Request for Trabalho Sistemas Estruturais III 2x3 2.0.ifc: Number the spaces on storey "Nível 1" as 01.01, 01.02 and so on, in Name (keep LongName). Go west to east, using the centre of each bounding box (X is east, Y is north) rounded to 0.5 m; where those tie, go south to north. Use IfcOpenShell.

First a look at what the model holds.

```python
import ifcopenshell
import ifcopenshell.util.element
import ifcopenshell.util.placement

model = ifcopenshell.open("Trabalho Sistemas Estruturais III 2x3 2.0.ifc")
print(model.schema)
storey = next(s for s in model.by_type("IfcBuildingStorey") if s.Name == "Nível 1")
spaces = [e for e in ifcopenshell.util.element.get_decomposition(storey) if e.is_a("IfcSpace")]
for e in sorted(spaces, key=lambda e: e.id()):
    origin = ifcopenshell.util.placement.get_local_placement(e.ObjectPlacement)[:3, 3]
    print(e.id(), e.Name, e.LongName, origin.round(2) + 0.0, sep=" | ")
```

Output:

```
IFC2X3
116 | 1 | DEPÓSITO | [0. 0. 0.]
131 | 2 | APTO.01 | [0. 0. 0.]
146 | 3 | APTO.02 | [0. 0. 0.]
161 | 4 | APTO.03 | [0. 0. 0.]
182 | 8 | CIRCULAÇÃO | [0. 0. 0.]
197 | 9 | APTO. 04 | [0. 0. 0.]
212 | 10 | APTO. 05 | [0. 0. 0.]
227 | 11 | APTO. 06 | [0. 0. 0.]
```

```python
import ifcopenshell
import ifcopenshell.geom
import ifcopenshell.util.element
import ifcopenshell.util.shape

model = ifcopenshell.open("Trabalho Sistemas Estruturais III 2x3 2.0.ifc")
settings = ifcopenshell.geom.settings()
settings.set("use-world-coords", True)


def centre(element):
    shape = ifcopenshell.geom.create_shape(settings, element)
    return ifcopenshell.util.shape.get_bbox_centroid(shape.geometry)


storey = next(s for s in model.by_type("IfcBuildingStorey") if s.Name == "Nível 1")
spaces = [e for e in ifcopenshell.util.element.get_decomposition(storey) if e.is_a("IfcSpace")]

# Insertion points can sit at a corner or the storey origin, so sort by the geometry (in metres).
centres = {e: centre(e) for e in spaces}
spaces.sort(key=lambda e: (round(centres[e][0] / 0.5), centres[e][1]))

for i, e in enumerate(spaces, start=1):
    number = f"01.{i:02d}"
    e.Name = number
    print(e.id(), number)

model.write("Trabalho Sistemas Estruturais III 2x3 2.0_rev.ifc")
```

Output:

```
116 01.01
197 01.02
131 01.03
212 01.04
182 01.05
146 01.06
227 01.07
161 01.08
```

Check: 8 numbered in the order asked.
